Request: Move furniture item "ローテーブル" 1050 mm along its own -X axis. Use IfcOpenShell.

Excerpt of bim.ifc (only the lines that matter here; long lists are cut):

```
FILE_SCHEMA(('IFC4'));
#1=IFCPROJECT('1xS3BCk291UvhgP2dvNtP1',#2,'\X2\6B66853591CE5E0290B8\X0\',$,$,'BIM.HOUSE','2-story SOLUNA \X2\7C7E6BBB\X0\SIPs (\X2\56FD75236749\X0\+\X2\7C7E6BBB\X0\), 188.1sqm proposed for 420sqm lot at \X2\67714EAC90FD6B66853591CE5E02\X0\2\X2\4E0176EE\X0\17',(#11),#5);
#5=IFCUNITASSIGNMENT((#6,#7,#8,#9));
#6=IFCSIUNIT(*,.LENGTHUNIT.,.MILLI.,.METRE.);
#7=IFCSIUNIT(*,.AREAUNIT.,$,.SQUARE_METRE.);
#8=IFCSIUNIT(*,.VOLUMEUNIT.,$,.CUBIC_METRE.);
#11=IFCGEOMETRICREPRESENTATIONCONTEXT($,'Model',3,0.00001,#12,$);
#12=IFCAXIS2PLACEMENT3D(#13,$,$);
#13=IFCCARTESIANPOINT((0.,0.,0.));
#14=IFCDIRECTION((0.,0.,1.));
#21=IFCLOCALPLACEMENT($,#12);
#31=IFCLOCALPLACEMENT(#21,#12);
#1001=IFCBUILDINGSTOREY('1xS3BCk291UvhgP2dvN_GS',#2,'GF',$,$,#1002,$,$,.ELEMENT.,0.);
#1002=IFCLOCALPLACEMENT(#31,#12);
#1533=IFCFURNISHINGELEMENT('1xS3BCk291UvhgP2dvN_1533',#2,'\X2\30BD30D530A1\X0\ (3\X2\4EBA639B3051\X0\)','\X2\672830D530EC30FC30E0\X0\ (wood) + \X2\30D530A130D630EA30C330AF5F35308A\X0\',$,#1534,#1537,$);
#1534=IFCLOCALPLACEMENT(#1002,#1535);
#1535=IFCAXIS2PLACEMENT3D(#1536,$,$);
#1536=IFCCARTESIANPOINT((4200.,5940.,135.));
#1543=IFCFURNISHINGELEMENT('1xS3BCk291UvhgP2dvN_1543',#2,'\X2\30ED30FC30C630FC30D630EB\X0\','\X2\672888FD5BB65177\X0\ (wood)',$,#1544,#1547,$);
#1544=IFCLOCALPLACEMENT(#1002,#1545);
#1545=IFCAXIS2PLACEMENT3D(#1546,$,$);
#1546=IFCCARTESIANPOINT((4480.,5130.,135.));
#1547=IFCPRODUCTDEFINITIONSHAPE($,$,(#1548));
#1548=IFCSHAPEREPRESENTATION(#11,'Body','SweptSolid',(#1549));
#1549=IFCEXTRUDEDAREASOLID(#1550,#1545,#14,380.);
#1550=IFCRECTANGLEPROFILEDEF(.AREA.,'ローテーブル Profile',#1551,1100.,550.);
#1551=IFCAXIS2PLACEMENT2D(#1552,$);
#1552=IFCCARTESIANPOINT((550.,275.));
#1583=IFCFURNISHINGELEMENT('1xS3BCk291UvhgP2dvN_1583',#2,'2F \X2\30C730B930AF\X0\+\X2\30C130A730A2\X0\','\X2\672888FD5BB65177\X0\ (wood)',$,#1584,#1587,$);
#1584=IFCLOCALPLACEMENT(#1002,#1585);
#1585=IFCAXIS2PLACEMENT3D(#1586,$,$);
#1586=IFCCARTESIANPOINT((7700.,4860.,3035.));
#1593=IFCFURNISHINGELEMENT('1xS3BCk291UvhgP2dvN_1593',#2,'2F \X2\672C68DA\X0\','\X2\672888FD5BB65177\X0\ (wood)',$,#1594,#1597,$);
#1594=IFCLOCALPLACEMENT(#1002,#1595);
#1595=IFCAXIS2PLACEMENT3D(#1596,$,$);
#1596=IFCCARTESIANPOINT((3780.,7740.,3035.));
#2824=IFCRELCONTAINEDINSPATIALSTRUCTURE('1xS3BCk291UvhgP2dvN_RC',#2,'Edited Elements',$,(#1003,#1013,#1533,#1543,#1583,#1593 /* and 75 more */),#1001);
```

```python
import ifcopenshell
import ifcopenshell.api.geometry
import ifcopenshell.util.placement
import ifcopenshell.util.unit

model = ifcopenshell.open("bim.ifc")
unit_scale = ifcopenshell.util.unit.calculate_unit_scale(model)

item = model.by_id(1543)
matrix = ifcopenshell.util.placement.get_local_placement(item.ObjectPlacement)
matrix[:3, 3] -= matrix[:3, 0] * 1.05 / unit_scale
ifcopenshell.api.geometry.edit_object_placement(model, product=item, matrix=matrix, is_si=False)

print(ifcopenshell.util.placement.get_local_placement(item.ObjectPlacement).round(3) + 0.0)

model.write("bim_updated.ifc")
```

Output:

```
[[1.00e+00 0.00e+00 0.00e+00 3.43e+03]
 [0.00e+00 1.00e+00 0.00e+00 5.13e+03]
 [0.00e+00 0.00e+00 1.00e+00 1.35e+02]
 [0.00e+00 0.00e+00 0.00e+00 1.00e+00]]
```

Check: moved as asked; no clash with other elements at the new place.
